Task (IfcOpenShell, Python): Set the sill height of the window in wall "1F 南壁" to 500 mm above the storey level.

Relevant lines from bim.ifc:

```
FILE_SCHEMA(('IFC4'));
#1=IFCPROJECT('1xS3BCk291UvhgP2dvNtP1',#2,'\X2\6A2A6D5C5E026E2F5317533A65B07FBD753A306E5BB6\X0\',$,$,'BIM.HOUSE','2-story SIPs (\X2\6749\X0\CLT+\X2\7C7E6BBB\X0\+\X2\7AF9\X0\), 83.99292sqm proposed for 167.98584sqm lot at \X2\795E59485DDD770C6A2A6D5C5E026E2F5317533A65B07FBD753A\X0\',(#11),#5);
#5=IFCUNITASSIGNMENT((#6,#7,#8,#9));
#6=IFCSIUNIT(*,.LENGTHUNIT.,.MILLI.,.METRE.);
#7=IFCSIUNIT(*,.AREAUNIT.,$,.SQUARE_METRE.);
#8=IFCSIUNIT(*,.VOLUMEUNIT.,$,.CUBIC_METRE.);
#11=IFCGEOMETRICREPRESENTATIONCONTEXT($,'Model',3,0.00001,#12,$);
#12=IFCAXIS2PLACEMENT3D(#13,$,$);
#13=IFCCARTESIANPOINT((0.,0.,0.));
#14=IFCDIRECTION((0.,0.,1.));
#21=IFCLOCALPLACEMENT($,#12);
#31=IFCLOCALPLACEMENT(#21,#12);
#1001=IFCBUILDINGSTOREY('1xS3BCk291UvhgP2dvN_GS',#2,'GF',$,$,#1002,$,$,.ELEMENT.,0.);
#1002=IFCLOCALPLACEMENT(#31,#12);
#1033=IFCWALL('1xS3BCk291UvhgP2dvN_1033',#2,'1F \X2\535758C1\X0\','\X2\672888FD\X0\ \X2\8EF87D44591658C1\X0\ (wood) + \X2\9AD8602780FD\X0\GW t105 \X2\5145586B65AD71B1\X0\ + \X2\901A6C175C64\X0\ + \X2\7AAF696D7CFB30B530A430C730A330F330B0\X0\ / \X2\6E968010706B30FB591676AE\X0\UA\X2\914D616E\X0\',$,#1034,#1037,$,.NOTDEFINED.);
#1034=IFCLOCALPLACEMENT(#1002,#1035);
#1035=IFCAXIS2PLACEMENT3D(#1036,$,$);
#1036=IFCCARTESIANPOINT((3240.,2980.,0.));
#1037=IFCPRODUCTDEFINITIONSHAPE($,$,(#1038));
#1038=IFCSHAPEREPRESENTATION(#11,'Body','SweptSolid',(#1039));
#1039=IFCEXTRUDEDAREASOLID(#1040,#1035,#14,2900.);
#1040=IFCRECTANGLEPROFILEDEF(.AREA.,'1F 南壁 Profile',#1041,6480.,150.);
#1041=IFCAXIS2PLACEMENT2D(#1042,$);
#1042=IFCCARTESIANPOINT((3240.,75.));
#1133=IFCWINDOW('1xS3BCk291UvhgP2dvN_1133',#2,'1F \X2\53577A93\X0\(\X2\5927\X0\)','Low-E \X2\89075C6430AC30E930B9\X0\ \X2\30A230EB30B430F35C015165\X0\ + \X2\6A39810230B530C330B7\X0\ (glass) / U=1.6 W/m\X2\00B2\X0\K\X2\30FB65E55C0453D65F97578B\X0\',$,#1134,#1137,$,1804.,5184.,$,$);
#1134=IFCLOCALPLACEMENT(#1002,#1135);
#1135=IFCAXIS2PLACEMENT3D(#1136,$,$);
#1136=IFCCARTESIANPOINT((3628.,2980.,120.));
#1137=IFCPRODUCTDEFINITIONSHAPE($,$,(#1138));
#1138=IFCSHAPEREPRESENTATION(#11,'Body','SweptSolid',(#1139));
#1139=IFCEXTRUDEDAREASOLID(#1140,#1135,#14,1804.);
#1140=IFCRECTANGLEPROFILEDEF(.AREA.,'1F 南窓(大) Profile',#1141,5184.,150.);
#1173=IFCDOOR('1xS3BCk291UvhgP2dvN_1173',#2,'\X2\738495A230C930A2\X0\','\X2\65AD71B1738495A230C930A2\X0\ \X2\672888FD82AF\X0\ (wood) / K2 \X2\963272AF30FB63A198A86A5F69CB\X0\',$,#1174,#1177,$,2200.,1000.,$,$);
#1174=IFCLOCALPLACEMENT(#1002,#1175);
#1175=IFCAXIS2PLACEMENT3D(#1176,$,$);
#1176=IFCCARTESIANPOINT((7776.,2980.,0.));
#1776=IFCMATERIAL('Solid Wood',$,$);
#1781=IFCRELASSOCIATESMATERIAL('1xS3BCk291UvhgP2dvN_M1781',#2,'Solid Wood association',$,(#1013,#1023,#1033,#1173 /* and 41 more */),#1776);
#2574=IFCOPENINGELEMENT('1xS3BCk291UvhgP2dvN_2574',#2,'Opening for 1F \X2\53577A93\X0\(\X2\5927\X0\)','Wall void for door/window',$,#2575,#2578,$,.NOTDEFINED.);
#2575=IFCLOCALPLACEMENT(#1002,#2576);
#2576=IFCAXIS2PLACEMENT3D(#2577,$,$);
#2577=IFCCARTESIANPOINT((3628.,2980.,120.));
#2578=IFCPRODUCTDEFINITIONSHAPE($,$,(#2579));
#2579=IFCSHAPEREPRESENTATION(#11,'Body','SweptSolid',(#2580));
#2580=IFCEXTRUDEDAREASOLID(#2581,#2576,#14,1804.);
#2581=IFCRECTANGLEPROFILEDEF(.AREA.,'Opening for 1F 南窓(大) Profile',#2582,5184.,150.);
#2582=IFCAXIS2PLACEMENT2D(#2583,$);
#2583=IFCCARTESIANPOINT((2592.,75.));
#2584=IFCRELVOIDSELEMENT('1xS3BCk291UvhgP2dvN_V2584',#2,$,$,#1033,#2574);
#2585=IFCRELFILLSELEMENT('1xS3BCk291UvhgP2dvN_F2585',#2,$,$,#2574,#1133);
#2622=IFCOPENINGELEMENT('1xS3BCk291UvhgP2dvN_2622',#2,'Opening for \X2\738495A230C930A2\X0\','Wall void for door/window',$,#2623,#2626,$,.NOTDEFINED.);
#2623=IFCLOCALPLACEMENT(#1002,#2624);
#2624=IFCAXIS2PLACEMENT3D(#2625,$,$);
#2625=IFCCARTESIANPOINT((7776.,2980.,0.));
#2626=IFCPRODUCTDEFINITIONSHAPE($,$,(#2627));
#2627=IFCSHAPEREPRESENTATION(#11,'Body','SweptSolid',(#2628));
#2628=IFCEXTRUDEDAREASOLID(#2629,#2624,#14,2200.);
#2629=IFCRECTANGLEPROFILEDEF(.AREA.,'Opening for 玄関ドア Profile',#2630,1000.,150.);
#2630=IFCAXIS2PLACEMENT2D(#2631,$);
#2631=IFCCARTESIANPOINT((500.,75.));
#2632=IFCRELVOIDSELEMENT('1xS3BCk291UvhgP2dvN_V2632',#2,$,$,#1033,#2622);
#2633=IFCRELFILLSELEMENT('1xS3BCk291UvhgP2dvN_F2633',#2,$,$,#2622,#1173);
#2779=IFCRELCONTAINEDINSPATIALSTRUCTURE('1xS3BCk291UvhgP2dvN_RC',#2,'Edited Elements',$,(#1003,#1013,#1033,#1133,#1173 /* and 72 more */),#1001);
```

```python
import numpy as np
import ifcopenshell
import ifcopenshell.api.geometry
import ifcopenshell.geom
import ifcopenshell.util.element
import ifcopenshell.util.placement
import ifcopenshell.util.shape
import ifcopenshell.util.unit

model = ifcopenshell.open("bim.ifc")
unit_scale = ifcopenshell.util.unit.calculate_unit_scale(model)

window = model.by_id(1133)
opening = window.FillsVoids[0].RelatingOpeningElement
storey = ifcopenshell.util.element.get_container(window, ifc_class="IfcBuildingStorey")
level = ifcopenshell.util.placement.get_local_placement(storey.ObjectPlacement)[2, 3]

# The opening's origin need not be at the sill, so measure its lowest point.
shape = ifcopenshell.geom.create_shape(ifcopenshell.geom.settings(), opening)
bottom = ifcopenshell.util.shape.get_shape_bottom_elevation(shape, shape.geometry) / unit_scale
dz = level + 500.0 - bottom

shift = np.array([0.0, 0.0, dz])
# The window is not placed relative to its opening, so move both.
for product in (opening, window):
    matrix = ifcopenshell.util.placement.get_local_placement(product.ObjectPlacement)
    matrix[:3, 3] += shift
    ifcopenshell.api.geometry.edit_object_placement(model, product=product, matrix=matrix, is_si=False)

print(f"moved by {dz * unit_scale:+.3f} m")

model.write("bim-out.ifc")
```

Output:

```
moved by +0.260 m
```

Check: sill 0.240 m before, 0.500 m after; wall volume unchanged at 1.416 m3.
